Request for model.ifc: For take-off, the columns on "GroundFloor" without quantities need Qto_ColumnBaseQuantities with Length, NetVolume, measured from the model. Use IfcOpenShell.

First a look at what the model holds.

```python
import ifcopenshell
import ifcopenshell.util.element
import ifcopenshell.util.unit

model = ifcopenshell.open("model.ifc")
print(model.schema)
for unit_type in ("LENGTHUNIT", "AREAUNIT", "VOLUMEUNIT"):
    print(unit_type, ifcopenshell.util.unit.calculate_unit_scale(model, unit_type))
storey = next(s for s in model.by_type("IfcBuildingStorey") if s.Name == "GroundFloor")
columns = [e for e in ifcopenshell.util.element.get_decomposition(storey) if e.is_a("IfcColumn")]
for e in sorted(columns, key=lambda e: e.id()):
    print(e.id(), e.is_a(), e.Name, list(ifcopenshell.util.element.get_psets(e, qtos_only=True)), sep=" | ")
```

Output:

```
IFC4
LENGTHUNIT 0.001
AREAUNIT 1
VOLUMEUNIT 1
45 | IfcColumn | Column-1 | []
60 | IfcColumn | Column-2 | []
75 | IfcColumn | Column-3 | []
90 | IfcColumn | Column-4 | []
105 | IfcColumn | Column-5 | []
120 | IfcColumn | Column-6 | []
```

```python
import ifcopenshell
import ifcopenshell.api.pset
import ifcopenshell.geom
import ifcopenshell.util.element
import ifcopenshell.util.shape
import ifcopenshell.util.unit

model = ifcopenshell.open("model.ifc")
unit_scale = ifcopenshell.util.unit.calculate_unit_scale(model)
volume_scale = ifcopenshell.util.unit.calculate_unit_scale(model, "VOLUMEUNIT")
settings = ifcopenshell.geom.settings()

storey = next(s for s in model.by_type("IfcBuildingStorey") if s.Name == "GroundFloor")
columns = [e for e in ifcopenshell.util.element.get_decomposition(storey) if e.is_a("IfcColumn")]

for e in sorted(columns, key=lambda e: e.id()):
    if ifcopenshell.util.element.get_psets(e, qtos_only=True, should_inherit=False):
        continue
    # Geometry comes back in metres, in the element's own axes.
    shape = ifcopenshell.geom.create_shape(settings, e)
    values = {
        "Length": ifcopenshell.util.shape.get_z(shape.geometry) / unit_scale,
        "NetVolume": ifcopenshell.util.shape.get_volume(shape.geometry) / volume_scale,
    }
    qto = ifcopenshell.api.pset.add_qto(model, product=e, name="Qto_ColumnBaseQuantities")
    ifcopenshell.api.pset.edit_qto(model, qto=qto, properties=values)
    print(e.id(), {k: round(v, 3) for k, v in values.items()})

model.write("model_updated.ifc")
```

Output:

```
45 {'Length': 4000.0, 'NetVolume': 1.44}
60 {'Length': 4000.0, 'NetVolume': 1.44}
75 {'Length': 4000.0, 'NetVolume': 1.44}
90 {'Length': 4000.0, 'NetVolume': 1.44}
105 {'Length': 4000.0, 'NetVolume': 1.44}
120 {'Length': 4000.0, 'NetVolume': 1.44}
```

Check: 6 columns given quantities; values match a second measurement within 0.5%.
